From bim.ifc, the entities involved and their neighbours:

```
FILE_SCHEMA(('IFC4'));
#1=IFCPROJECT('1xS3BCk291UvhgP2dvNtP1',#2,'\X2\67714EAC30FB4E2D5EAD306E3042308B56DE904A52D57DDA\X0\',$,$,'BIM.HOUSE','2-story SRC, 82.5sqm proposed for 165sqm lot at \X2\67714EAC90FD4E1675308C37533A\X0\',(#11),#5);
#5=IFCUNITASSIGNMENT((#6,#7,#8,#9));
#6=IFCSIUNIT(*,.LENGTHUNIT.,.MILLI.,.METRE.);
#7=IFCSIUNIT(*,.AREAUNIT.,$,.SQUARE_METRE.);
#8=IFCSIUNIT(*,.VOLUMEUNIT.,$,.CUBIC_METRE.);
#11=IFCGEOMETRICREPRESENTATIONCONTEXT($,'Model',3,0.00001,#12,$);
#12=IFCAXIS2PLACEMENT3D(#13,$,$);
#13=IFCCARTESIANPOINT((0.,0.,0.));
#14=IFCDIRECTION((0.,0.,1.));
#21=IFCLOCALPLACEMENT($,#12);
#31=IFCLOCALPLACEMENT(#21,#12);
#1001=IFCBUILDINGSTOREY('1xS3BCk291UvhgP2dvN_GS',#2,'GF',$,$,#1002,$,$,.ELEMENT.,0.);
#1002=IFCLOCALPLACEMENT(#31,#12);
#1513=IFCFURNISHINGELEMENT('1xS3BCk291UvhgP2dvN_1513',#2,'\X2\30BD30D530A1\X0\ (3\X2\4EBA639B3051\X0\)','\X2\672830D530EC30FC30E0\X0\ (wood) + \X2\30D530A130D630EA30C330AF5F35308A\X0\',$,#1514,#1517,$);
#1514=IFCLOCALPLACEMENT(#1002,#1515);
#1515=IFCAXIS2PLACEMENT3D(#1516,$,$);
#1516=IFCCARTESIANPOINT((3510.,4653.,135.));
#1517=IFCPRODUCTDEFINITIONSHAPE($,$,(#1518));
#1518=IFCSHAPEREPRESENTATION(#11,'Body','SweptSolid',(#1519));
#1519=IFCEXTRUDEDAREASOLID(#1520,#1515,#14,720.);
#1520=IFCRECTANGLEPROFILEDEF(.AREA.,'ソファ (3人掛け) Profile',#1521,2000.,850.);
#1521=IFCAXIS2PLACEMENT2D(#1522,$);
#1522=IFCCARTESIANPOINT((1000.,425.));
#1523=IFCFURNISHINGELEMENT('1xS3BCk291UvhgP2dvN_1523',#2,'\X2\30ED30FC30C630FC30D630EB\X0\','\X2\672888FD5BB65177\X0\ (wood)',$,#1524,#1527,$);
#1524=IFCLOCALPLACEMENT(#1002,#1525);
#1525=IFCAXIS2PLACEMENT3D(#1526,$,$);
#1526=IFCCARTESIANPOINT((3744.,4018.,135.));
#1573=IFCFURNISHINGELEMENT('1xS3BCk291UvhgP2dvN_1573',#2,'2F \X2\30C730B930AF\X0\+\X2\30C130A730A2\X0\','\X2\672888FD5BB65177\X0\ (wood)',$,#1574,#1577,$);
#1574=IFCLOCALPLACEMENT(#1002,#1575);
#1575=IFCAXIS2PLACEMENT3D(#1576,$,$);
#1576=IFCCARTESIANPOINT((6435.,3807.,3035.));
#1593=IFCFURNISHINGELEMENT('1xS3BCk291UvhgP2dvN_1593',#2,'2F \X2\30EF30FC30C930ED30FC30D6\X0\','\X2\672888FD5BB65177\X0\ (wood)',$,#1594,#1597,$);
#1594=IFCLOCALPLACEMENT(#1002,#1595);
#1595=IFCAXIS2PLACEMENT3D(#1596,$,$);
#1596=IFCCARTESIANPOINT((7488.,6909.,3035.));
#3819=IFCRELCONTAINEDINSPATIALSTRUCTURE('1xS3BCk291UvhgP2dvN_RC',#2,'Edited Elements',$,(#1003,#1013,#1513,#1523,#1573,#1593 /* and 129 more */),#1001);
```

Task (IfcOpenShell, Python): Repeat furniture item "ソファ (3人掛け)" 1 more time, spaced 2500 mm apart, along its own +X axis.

```python
import ifcopenshell
import ifcopenshell.api.geometry
import ifcopenshell.api.root
import ifcopenshell.util.element
import ifcopenshell.util.placement
import ifcopenshell.util.unit

model = ifcopenshell.open("bim.ifc")
unit_scale = ifcopenshell.util.unit.calculate_unit_scale(model)


def reuse_history(source, copy):
    """copy_class also copies each property set's owner history, people and application; keep the originals."""
    for rel in copy.IsDefinedBy:
        if rel.is_a("IfcRelDefinesByProperties") and (history := rel.RelatingPropertyDefinition.OwnerHistory):
            rel.RelatingPropertyDefinition.OwnerHistory = source.OwnerHistory
            ifcopenshell.util.element.remove_deep2(model, history)


source = model.by_guid("1xS3BCk291UvhgP2dvN_1513")
base = ifcopenshell.util.placement.get_local_placement(source.ObjectPlacement)
step = base[:3, 0] * 2.5 / unit_scale

for i in range(1, 2):
    copy = ifcopenshell.api.root.copy_class(model, product=source)
    copy.Representation = ifcopenshell.util.element.copy_deep(
        model, source.Representation, exclude=["IfcGeometricRepresentationContext", "IfcRepresentationMap"]
    )
    reuse_history(source, copy)
    matrix = base.copy()
    matrix[:3, 3] += i * step
    print("added at", matrix[:3, 3].round(3) + 0.0)
    ifcopenshell.api.geometry.edit_object_placement(model, product=copy, matrix=matrix, is_si=False)

model.write("bim_rev.ifc")
```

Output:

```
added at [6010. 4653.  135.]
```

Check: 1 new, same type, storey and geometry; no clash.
